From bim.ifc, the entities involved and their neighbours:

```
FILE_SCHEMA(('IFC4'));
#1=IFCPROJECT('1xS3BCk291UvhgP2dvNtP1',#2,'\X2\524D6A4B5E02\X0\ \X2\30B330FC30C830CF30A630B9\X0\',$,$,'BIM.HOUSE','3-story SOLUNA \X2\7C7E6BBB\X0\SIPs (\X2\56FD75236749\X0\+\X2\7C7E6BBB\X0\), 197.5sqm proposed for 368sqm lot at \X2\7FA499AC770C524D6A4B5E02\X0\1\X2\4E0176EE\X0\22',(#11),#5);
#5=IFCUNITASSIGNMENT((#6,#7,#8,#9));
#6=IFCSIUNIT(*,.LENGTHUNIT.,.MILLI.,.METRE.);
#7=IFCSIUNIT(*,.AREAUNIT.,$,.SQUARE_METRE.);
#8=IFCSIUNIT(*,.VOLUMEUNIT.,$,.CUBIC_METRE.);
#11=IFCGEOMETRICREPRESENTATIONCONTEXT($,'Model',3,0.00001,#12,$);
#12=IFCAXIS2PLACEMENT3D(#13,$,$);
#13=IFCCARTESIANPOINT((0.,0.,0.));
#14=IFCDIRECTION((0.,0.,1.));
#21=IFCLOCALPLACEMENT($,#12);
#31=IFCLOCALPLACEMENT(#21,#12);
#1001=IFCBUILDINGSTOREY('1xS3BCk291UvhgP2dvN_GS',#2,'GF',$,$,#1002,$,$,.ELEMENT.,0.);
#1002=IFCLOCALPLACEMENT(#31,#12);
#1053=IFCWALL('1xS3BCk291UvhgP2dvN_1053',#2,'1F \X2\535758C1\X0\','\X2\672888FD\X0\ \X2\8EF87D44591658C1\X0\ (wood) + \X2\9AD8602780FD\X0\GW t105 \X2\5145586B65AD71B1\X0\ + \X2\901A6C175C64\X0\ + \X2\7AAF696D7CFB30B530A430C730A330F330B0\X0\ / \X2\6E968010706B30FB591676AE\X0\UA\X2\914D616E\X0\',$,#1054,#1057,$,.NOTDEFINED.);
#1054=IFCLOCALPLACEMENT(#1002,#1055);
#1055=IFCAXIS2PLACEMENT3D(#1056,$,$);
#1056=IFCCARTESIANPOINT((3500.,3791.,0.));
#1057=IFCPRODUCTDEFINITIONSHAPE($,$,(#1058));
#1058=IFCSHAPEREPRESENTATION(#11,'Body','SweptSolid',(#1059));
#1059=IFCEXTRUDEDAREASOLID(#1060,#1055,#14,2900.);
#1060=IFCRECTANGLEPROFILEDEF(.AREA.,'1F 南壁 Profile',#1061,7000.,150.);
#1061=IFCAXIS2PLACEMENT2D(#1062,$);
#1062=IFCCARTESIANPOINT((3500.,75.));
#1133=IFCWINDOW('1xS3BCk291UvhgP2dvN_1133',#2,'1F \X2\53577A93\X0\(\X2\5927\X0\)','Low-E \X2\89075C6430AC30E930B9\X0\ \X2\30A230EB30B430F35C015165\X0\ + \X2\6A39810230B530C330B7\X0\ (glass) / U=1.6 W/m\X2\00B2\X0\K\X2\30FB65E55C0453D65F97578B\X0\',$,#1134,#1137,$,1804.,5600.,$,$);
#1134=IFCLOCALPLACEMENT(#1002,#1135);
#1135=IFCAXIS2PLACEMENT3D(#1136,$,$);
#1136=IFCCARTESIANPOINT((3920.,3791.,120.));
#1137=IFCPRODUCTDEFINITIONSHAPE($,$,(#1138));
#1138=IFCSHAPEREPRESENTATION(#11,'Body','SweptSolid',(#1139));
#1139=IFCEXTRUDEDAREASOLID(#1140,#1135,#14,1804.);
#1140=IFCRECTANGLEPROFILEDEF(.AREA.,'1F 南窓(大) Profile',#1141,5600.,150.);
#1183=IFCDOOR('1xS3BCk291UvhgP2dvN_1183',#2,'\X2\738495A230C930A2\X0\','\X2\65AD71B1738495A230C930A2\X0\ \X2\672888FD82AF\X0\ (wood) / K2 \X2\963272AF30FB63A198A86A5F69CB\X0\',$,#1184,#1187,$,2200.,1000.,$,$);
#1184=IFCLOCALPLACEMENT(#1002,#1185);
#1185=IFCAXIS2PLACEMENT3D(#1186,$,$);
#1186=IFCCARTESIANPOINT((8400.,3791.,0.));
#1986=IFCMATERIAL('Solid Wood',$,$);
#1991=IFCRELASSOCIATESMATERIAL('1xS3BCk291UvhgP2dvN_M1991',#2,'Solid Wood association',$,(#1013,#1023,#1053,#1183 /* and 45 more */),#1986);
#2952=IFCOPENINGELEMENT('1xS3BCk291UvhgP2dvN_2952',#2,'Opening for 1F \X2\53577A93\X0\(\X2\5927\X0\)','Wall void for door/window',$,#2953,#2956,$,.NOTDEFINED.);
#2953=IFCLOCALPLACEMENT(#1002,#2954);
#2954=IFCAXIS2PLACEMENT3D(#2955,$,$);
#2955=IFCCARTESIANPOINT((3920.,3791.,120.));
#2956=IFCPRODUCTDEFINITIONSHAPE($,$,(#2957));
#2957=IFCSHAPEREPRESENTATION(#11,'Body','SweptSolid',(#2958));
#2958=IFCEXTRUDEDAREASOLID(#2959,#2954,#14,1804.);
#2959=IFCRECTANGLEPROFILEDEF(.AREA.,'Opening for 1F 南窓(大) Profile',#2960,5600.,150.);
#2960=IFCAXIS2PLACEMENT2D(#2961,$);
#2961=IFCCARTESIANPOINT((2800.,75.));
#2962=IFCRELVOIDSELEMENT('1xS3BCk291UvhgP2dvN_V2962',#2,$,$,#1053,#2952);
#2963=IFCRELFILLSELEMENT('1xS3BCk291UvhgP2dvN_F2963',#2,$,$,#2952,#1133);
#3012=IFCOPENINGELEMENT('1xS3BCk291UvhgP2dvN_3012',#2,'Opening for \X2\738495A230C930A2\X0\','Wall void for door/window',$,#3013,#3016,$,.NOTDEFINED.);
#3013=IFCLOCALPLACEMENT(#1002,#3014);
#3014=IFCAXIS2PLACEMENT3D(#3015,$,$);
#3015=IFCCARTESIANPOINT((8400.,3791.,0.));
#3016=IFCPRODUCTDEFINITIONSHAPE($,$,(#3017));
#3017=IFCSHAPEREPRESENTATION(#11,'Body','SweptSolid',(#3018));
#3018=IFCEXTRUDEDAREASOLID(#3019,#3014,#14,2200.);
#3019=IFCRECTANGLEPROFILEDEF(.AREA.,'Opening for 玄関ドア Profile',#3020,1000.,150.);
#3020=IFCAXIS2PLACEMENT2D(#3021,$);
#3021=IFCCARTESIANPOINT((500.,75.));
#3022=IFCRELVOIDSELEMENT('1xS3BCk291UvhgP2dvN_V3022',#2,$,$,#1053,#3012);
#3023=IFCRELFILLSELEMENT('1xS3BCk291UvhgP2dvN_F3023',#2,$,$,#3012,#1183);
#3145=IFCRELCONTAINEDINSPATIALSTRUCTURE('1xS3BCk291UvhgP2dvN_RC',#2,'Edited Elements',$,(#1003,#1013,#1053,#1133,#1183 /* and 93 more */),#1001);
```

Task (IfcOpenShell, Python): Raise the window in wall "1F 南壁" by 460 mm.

```python
import numpy as np
import ifcopenshell
import ifcopenshell.api.geometry
import ifcopenshell.util.placement
import ifcopenshell.util.unit

model = ifcopenshell.open("bim.ifc")
unit_scale = ifcopenshell.util.unit.calculate_unit_scale(model)

window = model.by_guid("1xS3BCk291UvhgP2dvN_1133")
opening = window.FillsVoids[0].RelatingOpeningElement
dz = 460.0

shift = np.array([0.0, 0.0, dz])
# The window is not placed relative to its opening, so move both.
for product in (opening, window):
    matrix = ifcopenshell.util.placement.get_local_placement(product.ObjectPlacement)
    matrix[:3, 3] += shift
    ifcopenshell.api.geometry.edit_object_placement(model, product=product, matrix=matrix, is_si=False)

print(f"moved by {dz * unit_scale:+.3f} m")

model.write("bim_edited.ifc")
```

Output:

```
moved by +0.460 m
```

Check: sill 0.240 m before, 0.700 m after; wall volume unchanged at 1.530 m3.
